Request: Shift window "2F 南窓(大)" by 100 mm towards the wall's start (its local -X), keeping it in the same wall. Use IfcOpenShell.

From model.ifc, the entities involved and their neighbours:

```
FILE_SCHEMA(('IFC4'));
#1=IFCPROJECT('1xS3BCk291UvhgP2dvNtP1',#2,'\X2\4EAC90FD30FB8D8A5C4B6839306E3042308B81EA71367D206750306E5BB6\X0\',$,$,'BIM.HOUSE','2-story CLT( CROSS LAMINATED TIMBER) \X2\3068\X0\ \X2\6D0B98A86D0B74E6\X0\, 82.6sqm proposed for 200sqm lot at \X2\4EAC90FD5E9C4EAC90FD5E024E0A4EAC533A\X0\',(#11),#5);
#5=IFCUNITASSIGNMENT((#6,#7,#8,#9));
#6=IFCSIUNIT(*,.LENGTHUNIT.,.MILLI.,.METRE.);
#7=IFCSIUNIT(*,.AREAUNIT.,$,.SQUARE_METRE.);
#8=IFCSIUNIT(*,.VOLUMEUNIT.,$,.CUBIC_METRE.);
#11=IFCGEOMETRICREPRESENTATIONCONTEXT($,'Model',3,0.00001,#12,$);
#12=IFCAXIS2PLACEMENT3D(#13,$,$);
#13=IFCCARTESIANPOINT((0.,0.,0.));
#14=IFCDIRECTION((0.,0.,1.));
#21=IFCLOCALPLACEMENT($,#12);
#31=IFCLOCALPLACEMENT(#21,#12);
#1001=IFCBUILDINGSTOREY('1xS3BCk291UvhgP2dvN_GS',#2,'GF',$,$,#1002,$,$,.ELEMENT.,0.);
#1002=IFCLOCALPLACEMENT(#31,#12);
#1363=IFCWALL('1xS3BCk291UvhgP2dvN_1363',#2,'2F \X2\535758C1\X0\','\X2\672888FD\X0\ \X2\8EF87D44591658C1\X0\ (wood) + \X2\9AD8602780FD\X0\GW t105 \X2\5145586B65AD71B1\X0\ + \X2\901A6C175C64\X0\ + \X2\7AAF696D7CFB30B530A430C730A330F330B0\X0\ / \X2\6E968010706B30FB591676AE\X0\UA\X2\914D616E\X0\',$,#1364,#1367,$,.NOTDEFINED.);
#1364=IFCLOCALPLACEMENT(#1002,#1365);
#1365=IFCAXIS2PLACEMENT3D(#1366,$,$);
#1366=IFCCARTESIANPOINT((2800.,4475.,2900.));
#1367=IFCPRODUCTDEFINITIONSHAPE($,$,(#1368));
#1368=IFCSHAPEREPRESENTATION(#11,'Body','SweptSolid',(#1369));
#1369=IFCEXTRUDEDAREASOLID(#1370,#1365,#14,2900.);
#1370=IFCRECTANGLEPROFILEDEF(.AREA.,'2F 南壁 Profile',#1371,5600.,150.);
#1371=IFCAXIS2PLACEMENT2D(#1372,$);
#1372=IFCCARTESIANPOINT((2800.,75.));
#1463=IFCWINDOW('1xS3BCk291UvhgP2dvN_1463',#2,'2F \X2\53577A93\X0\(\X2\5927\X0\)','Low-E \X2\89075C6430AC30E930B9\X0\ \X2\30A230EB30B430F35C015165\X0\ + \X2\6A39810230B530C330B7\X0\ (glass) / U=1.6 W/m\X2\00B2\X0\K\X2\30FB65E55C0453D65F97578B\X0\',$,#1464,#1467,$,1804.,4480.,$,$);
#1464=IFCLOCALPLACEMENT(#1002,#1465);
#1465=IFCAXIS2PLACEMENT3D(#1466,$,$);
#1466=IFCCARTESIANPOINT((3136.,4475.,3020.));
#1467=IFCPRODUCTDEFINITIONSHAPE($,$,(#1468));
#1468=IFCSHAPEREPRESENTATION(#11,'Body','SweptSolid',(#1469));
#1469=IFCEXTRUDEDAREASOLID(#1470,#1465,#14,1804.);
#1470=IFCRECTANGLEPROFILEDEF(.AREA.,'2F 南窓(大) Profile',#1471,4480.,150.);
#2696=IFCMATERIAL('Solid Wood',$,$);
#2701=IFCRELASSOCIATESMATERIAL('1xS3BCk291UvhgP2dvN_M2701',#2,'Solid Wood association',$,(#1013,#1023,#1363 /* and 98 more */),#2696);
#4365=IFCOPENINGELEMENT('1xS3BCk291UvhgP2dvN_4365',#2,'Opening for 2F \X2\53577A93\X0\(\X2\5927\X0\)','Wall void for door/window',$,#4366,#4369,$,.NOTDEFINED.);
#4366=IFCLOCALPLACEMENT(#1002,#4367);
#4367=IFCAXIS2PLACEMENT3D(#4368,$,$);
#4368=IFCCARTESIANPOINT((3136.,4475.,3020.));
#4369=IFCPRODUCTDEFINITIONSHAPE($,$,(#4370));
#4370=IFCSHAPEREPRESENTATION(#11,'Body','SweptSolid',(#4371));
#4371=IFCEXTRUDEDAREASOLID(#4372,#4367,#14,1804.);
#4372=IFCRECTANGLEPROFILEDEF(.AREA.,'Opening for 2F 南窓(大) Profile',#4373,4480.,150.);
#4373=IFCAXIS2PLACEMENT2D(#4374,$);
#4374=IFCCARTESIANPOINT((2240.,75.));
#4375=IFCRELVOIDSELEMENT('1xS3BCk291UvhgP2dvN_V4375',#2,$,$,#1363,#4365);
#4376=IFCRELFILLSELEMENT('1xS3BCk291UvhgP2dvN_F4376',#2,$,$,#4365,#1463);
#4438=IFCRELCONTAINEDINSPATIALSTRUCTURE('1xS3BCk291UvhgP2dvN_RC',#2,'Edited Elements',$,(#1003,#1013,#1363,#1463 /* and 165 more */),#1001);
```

```python
import ifcopenshell
import ifcopenshell.api.geometry
import ifcopenshell.util.placement

model = ifcopenshell.open("model.ifc")

window = model.by_guid("1xS3BCk291UvhgP2dvN_1463")
opening = window.FillsVoids[0].RelatingOpeningElement
wall = opening.VoidsElements[0].RelatingBuildingElement

wall_matrix = ifcopenshell.util.placement.get_local_placement(wall.ObjectPlacement)
shift = wall_matrix[:3, 0] * -100.0
before = ifcopenshell.util.placement.get_local_placement(window.ObjectPlacement)[:3, 3].copy()

# The window is not placed relative to its opening, so move both.
for product in (opening, window):
    matrix = ifcopenshell.util.placement.get_local_placement(product.ObjectPlacement)
    matrix[:3, 3] += shift
    ifcopenshell.api.geometry.edit_object_placement(model, product=product, matrix=matrix, is_si=False)

after = ifcopenshell.util.placement.get_local_placement(window.ObjectPlacement)[:3, 3]
print("window moved by", (after - before).round(3) + 0.0)

model.write("model_v2.ifc")
```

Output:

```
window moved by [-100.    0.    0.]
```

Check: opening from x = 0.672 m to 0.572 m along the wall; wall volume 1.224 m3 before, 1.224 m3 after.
